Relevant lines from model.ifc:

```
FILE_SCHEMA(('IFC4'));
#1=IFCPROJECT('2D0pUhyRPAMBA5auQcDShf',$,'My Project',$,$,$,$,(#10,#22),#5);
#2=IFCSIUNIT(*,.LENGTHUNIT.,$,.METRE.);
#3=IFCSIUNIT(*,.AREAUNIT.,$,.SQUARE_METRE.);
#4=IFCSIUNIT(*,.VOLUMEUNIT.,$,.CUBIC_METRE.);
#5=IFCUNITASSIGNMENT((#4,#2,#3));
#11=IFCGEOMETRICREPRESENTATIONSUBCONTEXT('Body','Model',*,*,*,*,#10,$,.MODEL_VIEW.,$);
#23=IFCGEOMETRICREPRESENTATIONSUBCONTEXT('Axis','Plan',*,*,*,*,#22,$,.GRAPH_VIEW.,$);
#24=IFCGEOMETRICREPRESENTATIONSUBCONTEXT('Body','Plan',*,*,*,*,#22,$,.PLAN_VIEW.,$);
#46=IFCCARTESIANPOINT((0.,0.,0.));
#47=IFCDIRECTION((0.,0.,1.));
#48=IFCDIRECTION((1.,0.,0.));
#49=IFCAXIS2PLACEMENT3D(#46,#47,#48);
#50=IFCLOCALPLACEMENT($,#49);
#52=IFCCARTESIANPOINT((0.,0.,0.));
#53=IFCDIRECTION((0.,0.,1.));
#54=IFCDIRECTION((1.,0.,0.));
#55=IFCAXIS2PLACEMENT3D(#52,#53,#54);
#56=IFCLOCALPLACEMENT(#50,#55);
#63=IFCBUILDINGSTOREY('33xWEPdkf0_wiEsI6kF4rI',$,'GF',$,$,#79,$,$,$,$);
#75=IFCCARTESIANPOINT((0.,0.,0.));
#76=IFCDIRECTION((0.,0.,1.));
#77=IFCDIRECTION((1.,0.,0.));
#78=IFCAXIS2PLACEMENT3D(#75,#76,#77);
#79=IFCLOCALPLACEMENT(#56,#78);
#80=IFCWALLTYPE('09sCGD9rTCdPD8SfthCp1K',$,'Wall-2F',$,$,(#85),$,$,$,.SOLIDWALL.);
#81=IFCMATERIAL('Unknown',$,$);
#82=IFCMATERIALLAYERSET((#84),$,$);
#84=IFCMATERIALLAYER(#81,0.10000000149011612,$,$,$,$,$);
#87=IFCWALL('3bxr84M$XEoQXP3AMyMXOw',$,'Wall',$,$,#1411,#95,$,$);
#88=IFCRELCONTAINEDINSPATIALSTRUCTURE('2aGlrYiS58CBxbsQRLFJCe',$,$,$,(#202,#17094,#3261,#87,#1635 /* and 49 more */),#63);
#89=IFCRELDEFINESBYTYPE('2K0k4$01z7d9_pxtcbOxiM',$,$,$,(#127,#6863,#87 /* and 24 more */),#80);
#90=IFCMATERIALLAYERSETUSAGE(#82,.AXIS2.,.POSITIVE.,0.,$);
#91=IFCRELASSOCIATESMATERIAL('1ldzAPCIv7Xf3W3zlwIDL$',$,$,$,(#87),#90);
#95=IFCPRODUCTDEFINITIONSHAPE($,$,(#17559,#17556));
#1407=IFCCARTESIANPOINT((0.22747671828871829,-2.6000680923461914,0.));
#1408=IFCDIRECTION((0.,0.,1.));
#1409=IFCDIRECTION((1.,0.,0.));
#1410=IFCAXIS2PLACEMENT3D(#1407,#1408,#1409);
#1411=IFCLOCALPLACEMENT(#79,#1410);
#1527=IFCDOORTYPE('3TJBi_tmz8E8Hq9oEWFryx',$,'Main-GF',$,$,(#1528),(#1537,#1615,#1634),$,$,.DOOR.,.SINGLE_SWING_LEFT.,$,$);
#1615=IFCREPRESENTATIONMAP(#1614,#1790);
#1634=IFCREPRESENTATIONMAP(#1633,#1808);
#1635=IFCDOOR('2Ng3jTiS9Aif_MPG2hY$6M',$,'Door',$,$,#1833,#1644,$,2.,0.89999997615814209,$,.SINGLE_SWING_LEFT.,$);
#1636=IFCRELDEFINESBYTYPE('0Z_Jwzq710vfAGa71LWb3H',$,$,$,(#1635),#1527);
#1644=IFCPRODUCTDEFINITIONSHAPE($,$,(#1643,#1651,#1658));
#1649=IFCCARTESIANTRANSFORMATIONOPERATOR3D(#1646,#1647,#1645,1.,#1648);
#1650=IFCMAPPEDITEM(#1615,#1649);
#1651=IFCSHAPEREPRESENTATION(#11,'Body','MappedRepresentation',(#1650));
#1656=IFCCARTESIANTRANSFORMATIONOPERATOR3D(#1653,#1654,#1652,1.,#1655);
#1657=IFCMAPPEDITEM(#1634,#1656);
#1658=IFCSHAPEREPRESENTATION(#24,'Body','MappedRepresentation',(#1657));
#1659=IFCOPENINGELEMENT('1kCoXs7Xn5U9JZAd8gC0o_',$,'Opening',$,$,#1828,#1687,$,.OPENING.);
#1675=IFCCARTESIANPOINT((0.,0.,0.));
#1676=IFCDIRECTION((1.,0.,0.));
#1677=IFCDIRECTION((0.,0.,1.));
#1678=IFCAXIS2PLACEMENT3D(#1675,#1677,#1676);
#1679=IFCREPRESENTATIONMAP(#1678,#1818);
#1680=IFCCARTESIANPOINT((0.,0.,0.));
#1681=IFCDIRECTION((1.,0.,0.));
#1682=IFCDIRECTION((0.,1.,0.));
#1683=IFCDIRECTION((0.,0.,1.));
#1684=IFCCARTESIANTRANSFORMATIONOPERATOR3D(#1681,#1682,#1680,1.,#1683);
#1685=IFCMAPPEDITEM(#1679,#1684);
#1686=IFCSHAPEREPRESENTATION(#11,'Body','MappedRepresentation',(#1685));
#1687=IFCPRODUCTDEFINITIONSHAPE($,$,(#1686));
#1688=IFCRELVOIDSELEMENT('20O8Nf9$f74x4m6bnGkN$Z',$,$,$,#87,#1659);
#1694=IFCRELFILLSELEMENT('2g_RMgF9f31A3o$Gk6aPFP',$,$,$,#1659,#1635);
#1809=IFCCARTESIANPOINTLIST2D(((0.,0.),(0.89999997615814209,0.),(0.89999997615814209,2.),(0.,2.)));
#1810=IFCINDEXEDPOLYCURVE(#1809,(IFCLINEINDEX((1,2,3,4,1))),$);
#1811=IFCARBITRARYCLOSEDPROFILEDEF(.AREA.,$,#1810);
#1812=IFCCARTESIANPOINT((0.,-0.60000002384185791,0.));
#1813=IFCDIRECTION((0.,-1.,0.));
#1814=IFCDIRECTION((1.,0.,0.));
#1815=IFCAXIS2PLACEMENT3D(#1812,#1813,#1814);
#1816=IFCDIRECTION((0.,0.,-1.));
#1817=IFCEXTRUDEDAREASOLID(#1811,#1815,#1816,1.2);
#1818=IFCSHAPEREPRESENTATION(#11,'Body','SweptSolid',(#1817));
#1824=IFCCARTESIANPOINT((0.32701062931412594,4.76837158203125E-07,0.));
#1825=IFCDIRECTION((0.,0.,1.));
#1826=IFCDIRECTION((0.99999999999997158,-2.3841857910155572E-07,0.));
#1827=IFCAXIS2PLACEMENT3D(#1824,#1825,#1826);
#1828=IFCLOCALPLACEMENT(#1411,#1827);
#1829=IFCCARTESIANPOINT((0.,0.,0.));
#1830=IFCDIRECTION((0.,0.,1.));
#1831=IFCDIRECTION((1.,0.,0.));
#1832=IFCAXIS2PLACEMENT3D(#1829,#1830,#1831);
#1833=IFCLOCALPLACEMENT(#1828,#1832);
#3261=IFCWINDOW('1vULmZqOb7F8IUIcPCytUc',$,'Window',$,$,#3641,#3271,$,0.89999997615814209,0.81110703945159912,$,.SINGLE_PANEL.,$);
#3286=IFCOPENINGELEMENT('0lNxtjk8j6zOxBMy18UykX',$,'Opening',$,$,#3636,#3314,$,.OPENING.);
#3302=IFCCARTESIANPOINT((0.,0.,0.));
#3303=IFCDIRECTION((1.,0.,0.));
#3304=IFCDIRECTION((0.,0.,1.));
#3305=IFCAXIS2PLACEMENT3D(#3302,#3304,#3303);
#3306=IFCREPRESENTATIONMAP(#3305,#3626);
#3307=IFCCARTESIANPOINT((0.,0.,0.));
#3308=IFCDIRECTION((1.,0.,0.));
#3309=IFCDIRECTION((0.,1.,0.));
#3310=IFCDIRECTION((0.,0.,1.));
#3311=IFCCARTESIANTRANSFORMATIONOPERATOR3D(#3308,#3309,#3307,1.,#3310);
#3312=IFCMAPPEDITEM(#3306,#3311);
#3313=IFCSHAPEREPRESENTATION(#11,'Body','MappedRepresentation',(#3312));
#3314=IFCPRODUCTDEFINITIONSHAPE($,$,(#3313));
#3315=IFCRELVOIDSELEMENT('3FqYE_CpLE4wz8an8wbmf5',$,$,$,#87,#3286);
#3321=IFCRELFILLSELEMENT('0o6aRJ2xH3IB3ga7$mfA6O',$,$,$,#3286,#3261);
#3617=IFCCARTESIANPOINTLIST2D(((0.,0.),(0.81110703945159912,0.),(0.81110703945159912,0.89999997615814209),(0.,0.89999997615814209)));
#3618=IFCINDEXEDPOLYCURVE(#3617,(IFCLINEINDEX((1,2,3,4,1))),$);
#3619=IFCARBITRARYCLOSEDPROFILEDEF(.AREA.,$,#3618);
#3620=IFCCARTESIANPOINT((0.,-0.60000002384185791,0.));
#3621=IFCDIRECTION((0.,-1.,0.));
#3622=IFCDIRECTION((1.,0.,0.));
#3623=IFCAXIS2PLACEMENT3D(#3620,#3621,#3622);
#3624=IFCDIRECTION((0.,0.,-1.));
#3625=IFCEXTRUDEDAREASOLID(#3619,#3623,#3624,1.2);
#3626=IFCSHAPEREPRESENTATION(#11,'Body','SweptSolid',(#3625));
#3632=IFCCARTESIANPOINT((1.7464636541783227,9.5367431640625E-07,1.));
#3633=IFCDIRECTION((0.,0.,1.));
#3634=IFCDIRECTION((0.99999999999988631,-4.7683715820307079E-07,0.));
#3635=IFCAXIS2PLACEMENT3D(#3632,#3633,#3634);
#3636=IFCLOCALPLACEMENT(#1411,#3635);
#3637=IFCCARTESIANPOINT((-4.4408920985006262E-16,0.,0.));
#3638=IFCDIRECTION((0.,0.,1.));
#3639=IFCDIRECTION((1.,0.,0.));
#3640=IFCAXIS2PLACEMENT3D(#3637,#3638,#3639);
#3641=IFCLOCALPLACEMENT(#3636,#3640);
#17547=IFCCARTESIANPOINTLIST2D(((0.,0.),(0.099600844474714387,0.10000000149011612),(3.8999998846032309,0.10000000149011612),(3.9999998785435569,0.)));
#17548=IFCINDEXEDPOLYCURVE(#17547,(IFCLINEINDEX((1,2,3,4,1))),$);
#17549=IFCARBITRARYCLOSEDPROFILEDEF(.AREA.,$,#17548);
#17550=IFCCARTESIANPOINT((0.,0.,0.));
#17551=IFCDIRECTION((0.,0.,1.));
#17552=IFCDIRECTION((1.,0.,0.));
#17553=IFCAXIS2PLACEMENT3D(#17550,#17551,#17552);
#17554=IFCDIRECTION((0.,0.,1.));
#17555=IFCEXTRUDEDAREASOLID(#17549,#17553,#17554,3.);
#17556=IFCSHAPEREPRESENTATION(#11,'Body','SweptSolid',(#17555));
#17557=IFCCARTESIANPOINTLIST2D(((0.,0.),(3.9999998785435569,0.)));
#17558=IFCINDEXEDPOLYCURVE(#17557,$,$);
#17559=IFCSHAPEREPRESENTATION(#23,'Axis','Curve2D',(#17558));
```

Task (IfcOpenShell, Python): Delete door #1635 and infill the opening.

```python
import ifcopenshell
import ifcopenshell.api.feature
import ifcopenshell.api.root
import ifcopenshell.geom
import ifcopenshell.util.shape

model = ifcopenshell.open("model.ifc")
settings = ifcopenshell.geom.settings()


def volume(element):
    """Net volume in cubic metres, openings subtracted."""
    shape = ifcopenshell.geom.create_shape(settings, element)
    return ifcopenshell.util.shape.get_volume(shape.geometry)


door = model.by_id(1635)
opening = door.FillsVoids[0].RelatingOpeningElement
wall = opening.VoidsElements[0].RelatingBuildingElement
before = volume(wall)

ifcopenshell.api.root.remove_product(model, product=door)
ifcopenshell.api.feature.remove_feature(model, feature=opening)

after = volume(wall)

print(f"wall volume {before:.3f} -> {after:.3f} m3")

model.write("model_updated.ifc")
```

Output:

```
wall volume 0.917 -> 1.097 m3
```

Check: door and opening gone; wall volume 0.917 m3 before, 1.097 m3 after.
